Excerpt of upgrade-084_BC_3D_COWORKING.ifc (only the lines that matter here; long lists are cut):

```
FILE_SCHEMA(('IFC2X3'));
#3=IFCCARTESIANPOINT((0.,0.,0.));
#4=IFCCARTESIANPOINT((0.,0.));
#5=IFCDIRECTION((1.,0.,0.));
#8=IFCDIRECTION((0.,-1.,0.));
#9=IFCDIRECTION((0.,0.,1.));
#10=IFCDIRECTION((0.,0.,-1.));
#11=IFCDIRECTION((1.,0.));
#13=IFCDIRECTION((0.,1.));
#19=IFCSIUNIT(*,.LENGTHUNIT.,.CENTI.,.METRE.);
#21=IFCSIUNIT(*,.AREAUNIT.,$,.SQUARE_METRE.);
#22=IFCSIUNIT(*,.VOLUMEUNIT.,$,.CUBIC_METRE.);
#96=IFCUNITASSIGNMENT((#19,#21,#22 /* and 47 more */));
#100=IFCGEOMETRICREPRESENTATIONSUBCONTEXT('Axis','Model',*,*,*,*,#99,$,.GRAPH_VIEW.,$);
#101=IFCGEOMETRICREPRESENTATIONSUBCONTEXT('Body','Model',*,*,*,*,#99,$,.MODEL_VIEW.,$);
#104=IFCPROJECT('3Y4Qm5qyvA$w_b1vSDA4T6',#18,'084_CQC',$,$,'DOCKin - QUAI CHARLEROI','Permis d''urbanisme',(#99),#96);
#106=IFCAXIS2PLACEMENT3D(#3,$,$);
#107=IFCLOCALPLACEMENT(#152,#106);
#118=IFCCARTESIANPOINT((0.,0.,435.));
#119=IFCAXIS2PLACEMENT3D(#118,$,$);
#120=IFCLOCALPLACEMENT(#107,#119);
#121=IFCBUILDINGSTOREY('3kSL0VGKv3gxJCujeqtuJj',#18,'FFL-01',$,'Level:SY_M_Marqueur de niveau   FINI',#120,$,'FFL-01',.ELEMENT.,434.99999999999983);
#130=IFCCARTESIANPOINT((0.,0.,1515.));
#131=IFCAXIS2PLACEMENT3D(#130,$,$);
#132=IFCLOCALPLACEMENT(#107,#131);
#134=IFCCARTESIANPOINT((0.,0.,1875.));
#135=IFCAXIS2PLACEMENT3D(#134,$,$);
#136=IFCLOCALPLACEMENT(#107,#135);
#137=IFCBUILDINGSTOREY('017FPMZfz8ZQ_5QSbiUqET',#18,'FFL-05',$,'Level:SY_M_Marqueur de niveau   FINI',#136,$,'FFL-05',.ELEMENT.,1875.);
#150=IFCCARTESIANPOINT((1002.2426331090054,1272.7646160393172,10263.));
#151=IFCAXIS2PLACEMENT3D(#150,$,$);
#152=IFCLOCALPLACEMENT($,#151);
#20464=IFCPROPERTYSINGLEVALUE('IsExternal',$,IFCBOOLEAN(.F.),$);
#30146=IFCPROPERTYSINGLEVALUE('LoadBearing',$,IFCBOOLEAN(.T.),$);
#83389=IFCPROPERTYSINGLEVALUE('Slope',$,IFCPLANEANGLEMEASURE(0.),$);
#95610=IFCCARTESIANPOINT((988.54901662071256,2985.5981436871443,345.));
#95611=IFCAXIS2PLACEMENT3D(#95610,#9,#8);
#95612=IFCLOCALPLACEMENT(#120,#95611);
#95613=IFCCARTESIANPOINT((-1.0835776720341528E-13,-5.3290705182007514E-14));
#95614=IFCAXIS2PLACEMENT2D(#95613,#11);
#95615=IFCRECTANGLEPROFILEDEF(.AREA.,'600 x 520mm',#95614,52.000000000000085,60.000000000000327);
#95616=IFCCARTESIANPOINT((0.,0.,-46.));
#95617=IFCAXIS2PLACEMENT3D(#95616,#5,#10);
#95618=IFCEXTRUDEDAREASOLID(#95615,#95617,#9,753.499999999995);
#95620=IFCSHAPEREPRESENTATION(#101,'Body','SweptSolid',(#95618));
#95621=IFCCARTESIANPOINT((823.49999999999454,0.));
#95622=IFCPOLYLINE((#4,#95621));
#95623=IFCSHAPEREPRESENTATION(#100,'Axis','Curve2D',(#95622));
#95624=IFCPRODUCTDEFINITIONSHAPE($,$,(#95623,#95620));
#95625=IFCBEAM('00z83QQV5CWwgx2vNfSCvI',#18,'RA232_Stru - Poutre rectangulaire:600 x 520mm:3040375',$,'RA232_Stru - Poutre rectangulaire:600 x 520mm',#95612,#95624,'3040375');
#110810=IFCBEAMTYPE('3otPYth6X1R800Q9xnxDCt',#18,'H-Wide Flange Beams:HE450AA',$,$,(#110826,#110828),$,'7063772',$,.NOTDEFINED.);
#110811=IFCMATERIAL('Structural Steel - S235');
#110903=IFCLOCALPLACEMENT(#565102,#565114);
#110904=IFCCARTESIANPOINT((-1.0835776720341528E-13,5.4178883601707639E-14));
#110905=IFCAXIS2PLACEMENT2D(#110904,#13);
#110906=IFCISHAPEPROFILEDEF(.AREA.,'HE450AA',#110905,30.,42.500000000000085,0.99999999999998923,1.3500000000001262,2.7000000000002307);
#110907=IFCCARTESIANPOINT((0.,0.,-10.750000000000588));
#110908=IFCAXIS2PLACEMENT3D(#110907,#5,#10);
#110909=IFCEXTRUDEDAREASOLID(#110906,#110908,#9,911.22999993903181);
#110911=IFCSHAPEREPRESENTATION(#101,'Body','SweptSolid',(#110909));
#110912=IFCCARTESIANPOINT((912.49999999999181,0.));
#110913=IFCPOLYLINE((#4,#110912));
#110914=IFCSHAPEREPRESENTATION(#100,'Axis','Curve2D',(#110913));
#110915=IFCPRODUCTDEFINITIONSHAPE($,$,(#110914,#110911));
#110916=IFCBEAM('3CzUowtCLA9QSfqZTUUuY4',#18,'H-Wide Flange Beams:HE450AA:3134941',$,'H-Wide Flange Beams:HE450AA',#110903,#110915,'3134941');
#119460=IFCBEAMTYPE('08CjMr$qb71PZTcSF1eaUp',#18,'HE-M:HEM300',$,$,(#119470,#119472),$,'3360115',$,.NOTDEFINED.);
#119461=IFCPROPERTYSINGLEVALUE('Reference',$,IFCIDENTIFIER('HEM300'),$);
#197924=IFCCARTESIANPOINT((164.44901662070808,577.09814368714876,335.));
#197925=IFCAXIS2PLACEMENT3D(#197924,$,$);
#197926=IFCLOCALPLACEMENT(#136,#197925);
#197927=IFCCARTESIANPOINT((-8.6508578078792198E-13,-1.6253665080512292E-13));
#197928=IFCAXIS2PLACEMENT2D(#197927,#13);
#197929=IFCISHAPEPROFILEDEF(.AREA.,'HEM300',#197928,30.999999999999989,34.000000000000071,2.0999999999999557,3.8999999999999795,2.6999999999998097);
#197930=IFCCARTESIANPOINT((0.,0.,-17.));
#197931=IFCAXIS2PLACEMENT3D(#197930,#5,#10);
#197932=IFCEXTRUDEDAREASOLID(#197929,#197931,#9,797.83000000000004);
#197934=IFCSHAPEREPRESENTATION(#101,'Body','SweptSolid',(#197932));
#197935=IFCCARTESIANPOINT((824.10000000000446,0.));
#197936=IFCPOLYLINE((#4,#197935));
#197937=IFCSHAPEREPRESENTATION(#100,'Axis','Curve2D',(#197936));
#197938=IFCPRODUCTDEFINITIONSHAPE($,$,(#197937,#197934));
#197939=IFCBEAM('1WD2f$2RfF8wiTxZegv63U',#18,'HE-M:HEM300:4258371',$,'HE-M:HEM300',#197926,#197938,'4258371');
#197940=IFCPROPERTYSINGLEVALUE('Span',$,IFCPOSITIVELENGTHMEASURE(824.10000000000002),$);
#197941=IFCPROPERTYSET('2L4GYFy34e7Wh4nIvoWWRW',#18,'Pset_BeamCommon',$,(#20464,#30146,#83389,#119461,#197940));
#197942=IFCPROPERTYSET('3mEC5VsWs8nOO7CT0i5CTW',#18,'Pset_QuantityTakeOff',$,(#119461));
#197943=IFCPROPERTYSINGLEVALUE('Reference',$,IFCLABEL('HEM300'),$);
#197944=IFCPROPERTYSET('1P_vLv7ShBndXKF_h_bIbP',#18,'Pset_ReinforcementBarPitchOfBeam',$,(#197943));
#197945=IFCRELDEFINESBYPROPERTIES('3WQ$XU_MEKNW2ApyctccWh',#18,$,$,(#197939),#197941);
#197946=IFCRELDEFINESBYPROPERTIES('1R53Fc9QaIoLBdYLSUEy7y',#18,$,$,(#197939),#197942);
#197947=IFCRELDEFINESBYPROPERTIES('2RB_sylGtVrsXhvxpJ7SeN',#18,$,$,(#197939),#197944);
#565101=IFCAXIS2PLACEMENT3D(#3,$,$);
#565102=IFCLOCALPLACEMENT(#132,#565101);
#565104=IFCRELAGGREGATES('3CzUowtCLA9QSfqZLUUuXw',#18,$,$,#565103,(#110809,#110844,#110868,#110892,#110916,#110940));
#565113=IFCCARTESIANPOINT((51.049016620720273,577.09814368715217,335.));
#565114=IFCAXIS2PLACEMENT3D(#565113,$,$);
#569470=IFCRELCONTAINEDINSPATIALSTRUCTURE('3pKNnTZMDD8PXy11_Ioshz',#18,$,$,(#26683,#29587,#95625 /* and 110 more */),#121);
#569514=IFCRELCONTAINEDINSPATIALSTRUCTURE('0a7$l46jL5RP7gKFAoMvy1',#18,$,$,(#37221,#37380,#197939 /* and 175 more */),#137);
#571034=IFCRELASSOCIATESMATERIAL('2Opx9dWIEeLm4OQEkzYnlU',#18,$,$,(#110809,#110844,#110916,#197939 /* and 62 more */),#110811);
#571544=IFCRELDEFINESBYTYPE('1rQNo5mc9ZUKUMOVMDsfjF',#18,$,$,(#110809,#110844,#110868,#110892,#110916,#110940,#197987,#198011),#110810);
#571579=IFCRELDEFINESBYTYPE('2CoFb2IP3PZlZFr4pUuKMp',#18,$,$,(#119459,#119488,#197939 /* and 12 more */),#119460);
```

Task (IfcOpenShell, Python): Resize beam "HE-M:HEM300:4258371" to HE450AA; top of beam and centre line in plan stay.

```python
import ifcopenshell
import ifcopenshell.api.pset
import ifcopenshell.api.type
import ifcopenshell.util.element
import ifcopenshell.util.representation

model = ifcopenshell.open("upgrade-084_BC_3D_COWORKING.ifc")

member = model.by_guid("1WD2f$2RfF8wiTxZegv63U")
source = next(p for p in model.by_type("IfcIShapeProfileDef") if p.ProfileName == "HE450AA")

body = ifcopenshell.util.representation.get_representation(member, "Model", "Body")
solid = body.Items[0]
old_profile = solid.SweptArea

# Copy the section's sizes but keep this member's own profile position.
profile = ifcopenshell.util.element.copy(model, source)
# Profiles are centred, so shift by half the change in depth to hold the top.
shift = (old_profile.OverallDepth - profile.OverallDepth) / 2
x, y = old_profile.Position.Location.Coordinates
up = (-1.0, 0.0)  # upwards, in the solid's own plane
location = model.createIfcCartesianPoint((x + up[0] * shift, y + up[1] * shift))
profile.Position = model.createIfcAxis2Placement2D(location, old_profile.Position.RefDirection)
solid.SweptArea = profile
if not model.get_total_inverses(old_profile):
    ifcopenshell.util.element.remove_deep2(model, old_profile)

new_type = model.by_guid("3otPYth6X1R800Q9xnxDCt")
ifcopenshell.api.type.assign_type(
    model, related_objects=[member], relating_type=new_type, should_map_representations=False
)
member.Name = member.Name.replace("HEM300", "HE450AA")
member.ObjectType = "HE-M:HE450AA"
pset = model.by_id(ifcopenshell.util.element.get_pset(member, "Pset_BeamCommon", should_inherit=False)["id"])
ifcopenshell.api.pset.edit_pset(model, pset=pset, properties={"Reference": "HE450AA"})
pset = model.by_id(ifcopenshell.util.element.get_pset(member, "Pset_QuantityTakeOff", should_inherit=False)["id"])
ifcopenshell.api.pset.edit_pset(model, pset=pset, properties={"Reference": "HE450AA"})
pset = model.by_id(ifcopenshell.util.element.get_pset(member, "Pset_ReinforcementBarPitchOfBeam", should_inherit=False)["id"])
ifcopenshell.api.pset.edit_pset(model, pset=pset, properties={"Reference": "HE450AA"})

print(solid.SweptArea)

model.write("upgrade-084_BC_3D_COWORKING_edited.ifc")
```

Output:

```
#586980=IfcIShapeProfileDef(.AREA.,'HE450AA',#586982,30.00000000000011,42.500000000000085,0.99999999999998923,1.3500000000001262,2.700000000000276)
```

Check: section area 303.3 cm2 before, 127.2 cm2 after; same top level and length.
